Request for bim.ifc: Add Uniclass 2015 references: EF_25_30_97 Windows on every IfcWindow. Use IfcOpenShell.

First a look at what the model holds.

```python
import ifcopenshell

model = ifcopenshell.open("bim.ifc")
print(model.schema)
print("classifications:", [c.Name for c in model.by_type("IfcClassification")])
for ifc_class in ("IfcDoor", "IfcRoof", "IfcStair", "IfcWall", "IfcWindow"):
    print(ifc_class, len(model.by_type(ifc_class)))
```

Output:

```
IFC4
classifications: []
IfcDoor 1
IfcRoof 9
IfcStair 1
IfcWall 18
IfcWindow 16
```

```python
import ifcopenshell
import ifcopenshell.api.classification

model = ifcopenshell.open("bim.ifc")

system = ifcopenshell.api.classification.add_classification(model, classification="Uniclass 2015")

codes = {
    "IfcWindow": ("EF_25_30_97", "Windows"),
}
for ifc_class, (code, name) in codes.items():
    products = model.by_type(ifc_class)
    ifcopenshell.api.classification.add_reference(
        model, products=products, classification=system, identification=code, name=name
    )
    print(code, len(products))

model.write("bim_edited.ifc")
```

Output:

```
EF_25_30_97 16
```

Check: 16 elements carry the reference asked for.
